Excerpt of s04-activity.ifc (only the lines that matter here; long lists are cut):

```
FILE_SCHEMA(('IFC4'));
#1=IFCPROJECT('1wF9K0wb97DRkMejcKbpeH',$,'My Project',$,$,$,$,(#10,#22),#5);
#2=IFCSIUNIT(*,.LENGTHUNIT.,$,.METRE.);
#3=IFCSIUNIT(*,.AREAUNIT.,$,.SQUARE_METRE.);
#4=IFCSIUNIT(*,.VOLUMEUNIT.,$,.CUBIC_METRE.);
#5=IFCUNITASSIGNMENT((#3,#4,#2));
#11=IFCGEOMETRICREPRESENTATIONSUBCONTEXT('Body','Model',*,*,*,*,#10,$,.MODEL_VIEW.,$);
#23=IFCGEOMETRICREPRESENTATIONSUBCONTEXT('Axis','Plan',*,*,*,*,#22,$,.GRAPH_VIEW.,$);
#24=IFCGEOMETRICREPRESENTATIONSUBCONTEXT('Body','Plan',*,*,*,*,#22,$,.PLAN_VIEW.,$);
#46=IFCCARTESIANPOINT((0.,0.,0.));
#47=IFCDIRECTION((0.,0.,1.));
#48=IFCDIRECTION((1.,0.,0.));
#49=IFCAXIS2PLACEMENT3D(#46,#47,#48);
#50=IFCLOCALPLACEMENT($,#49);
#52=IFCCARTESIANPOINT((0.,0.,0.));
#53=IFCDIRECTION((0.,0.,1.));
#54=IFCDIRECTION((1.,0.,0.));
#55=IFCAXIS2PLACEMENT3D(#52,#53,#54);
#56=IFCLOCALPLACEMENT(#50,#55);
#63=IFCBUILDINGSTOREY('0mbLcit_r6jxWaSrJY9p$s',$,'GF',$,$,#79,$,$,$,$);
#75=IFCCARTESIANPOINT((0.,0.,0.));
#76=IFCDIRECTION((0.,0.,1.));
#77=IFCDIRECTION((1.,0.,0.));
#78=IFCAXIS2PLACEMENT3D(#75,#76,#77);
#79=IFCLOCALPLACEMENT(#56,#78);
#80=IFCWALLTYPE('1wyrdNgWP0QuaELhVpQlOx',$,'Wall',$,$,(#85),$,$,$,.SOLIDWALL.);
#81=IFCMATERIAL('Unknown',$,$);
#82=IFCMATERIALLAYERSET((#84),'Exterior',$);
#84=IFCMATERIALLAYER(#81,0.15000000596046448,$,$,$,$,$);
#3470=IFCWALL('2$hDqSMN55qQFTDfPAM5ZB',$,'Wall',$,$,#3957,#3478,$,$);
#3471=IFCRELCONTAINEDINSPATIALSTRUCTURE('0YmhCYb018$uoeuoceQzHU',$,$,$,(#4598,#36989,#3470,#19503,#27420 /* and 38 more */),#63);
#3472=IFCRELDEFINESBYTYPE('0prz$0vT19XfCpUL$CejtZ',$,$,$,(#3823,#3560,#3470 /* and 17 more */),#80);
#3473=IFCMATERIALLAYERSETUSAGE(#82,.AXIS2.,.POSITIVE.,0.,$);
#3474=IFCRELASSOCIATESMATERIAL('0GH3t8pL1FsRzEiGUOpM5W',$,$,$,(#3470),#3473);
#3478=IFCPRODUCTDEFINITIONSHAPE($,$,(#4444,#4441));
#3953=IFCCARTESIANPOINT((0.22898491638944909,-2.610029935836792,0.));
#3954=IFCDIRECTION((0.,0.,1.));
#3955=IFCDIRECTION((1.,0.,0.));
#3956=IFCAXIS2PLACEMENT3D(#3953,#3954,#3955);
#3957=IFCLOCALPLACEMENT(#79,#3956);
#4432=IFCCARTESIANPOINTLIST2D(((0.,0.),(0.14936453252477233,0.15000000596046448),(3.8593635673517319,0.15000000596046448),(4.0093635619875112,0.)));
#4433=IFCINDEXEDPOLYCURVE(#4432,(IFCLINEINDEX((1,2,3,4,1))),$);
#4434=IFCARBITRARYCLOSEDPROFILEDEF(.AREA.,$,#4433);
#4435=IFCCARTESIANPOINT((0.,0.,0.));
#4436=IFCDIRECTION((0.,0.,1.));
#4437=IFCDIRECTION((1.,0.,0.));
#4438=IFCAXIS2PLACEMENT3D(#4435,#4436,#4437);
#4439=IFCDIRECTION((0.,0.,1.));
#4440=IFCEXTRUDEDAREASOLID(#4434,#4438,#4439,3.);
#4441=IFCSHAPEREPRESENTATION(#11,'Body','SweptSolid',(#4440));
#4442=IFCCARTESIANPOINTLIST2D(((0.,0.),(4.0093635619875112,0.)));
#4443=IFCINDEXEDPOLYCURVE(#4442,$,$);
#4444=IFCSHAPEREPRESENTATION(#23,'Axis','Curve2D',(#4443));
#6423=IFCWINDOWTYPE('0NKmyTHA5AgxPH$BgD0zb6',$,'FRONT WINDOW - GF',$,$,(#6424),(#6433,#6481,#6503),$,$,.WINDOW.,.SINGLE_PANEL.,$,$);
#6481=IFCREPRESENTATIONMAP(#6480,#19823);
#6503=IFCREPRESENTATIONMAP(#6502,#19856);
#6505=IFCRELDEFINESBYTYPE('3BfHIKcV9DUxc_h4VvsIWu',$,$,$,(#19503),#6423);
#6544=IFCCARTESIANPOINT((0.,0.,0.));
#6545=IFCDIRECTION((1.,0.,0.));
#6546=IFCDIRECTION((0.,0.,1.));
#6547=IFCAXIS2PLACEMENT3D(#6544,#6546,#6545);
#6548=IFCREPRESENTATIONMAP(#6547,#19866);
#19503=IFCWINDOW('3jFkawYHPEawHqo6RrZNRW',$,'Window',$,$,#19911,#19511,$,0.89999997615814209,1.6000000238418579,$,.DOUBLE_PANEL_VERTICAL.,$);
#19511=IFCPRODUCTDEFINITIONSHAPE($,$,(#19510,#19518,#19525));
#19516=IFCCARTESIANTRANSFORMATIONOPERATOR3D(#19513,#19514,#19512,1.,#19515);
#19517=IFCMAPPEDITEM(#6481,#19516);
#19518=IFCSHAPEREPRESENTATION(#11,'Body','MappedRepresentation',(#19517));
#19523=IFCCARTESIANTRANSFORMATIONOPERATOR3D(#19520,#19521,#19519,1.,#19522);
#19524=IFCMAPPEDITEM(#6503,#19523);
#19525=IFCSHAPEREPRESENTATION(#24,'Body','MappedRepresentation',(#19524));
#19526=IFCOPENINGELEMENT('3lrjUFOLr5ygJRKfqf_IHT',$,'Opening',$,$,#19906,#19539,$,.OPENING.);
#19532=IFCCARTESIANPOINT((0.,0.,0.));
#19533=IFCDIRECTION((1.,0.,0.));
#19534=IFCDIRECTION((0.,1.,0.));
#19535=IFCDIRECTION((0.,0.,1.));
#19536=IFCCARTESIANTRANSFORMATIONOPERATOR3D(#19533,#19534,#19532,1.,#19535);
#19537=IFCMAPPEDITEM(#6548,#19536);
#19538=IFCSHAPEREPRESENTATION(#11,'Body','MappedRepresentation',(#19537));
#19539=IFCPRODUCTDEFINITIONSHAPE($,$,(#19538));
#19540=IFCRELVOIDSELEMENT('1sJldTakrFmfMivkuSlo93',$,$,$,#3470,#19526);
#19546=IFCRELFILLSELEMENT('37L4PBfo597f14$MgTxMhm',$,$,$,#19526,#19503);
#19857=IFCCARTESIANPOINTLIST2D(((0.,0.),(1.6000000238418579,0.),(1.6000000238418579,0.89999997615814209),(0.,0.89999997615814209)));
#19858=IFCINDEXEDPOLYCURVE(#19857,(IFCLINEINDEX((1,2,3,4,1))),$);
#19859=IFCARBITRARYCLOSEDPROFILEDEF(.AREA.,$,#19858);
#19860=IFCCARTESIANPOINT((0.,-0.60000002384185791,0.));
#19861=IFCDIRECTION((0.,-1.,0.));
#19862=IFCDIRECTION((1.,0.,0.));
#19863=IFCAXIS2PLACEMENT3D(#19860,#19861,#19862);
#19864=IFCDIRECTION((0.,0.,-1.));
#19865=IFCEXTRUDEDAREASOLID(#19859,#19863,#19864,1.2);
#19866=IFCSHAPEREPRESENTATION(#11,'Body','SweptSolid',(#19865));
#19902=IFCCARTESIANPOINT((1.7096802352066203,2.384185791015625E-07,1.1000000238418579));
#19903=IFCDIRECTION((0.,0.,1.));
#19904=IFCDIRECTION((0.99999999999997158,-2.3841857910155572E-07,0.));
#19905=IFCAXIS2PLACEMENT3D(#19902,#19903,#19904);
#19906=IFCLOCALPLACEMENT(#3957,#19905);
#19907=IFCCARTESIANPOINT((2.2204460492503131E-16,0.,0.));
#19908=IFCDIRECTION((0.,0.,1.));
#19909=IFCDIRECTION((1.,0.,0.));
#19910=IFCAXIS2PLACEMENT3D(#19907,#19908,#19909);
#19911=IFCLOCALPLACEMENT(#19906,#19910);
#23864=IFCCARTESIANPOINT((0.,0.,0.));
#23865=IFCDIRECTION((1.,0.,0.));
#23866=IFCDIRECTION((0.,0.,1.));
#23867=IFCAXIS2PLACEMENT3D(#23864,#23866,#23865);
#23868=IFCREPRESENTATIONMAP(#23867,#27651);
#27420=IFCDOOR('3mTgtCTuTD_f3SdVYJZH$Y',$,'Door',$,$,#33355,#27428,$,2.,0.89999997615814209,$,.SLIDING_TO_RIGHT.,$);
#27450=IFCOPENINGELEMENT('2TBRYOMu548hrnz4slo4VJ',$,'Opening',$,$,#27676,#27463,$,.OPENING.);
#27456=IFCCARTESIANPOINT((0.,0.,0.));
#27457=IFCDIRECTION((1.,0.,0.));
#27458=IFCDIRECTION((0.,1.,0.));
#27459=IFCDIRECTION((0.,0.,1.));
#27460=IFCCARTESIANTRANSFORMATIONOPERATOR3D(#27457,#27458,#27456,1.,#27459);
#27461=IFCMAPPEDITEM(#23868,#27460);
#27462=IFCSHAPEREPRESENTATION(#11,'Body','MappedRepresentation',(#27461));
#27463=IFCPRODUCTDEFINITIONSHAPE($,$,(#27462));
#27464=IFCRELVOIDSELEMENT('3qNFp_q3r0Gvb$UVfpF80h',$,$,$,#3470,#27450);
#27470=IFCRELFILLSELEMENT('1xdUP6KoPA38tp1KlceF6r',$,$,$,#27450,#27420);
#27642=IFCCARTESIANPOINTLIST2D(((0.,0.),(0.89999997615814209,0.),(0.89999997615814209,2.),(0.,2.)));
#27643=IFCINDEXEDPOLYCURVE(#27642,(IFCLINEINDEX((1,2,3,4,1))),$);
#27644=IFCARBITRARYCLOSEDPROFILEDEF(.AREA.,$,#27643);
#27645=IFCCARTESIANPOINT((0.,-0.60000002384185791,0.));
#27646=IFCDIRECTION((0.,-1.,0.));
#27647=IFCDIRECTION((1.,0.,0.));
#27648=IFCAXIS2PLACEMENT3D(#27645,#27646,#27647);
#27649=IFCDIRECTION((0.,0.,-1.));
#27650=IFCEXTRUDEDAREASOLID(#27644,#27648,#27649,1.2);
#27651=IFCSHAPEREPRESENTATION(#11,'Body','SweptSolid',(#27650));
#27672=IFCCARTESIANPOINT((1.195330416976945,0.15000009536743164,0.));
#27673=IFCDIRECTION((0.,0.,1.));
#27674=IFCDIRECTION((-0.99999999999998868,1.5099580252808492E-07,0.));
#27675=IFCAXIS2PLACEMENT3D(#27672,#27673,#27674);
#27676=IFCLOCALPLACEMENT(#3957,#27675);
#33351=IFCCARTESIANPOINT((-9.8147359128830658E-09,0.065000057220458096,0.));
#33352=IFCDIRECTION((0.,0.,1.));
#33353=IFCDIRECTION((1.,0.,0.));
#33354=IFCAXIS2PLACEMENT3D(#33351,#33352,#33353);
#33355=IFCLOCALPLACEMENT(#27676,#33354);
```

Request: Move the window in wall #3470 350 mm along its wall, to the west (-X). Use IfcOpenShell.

```python
import ifcopenshell
import ifcopenshell.api.geometry
import ifcopenshell.util.placement
import ifcopenshell.util.unit

model = ifcopenshell.open("s04-activity.ifc")
unit_scale = ifcopenshell.util.unit.calculate_unit_scale(model)

window = model.by_guid("3jFkawYHPEawHqo6RrZNRW")
opening = window.FillsVoids[0].RelatingOpeningElement
wall = opening.VoidsElements[0].RelatingBuildingElement

wall_matrix = ifcopenshell.util.placement.get_local_placement(wall.ObjectPlacement)
shift = wall_matrix[:3, 0] * -0.35 / unit_scale
before = ifcopenshell.util.placement.get_local_placement(window.ObjectPlacement)[:3, 3].copy()

# The window is placed relative to its opening, so it follows when the opening moves.
matrix = ifcopenshell.util.placement.get_local_placement(opening.ObjectPlacement)
matrix[:3, 3] += shift
ifcopenshell.api.geometry.edit_object_placement(
    model, product=opening, matrix=matrix, is_si=False, should_transform_children=True
)

after = ifcopenshell.util.placement.get_local_placement(window.ObjectPlacement)[:3, 3]
print("window moved by", (after - before).round(3) + 0.0)

model.write("s04-activity_edited.ifc")
```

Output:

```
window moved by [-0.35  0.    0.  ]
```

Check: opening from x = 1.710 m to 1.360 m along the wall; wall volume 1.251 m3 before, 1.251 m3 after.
